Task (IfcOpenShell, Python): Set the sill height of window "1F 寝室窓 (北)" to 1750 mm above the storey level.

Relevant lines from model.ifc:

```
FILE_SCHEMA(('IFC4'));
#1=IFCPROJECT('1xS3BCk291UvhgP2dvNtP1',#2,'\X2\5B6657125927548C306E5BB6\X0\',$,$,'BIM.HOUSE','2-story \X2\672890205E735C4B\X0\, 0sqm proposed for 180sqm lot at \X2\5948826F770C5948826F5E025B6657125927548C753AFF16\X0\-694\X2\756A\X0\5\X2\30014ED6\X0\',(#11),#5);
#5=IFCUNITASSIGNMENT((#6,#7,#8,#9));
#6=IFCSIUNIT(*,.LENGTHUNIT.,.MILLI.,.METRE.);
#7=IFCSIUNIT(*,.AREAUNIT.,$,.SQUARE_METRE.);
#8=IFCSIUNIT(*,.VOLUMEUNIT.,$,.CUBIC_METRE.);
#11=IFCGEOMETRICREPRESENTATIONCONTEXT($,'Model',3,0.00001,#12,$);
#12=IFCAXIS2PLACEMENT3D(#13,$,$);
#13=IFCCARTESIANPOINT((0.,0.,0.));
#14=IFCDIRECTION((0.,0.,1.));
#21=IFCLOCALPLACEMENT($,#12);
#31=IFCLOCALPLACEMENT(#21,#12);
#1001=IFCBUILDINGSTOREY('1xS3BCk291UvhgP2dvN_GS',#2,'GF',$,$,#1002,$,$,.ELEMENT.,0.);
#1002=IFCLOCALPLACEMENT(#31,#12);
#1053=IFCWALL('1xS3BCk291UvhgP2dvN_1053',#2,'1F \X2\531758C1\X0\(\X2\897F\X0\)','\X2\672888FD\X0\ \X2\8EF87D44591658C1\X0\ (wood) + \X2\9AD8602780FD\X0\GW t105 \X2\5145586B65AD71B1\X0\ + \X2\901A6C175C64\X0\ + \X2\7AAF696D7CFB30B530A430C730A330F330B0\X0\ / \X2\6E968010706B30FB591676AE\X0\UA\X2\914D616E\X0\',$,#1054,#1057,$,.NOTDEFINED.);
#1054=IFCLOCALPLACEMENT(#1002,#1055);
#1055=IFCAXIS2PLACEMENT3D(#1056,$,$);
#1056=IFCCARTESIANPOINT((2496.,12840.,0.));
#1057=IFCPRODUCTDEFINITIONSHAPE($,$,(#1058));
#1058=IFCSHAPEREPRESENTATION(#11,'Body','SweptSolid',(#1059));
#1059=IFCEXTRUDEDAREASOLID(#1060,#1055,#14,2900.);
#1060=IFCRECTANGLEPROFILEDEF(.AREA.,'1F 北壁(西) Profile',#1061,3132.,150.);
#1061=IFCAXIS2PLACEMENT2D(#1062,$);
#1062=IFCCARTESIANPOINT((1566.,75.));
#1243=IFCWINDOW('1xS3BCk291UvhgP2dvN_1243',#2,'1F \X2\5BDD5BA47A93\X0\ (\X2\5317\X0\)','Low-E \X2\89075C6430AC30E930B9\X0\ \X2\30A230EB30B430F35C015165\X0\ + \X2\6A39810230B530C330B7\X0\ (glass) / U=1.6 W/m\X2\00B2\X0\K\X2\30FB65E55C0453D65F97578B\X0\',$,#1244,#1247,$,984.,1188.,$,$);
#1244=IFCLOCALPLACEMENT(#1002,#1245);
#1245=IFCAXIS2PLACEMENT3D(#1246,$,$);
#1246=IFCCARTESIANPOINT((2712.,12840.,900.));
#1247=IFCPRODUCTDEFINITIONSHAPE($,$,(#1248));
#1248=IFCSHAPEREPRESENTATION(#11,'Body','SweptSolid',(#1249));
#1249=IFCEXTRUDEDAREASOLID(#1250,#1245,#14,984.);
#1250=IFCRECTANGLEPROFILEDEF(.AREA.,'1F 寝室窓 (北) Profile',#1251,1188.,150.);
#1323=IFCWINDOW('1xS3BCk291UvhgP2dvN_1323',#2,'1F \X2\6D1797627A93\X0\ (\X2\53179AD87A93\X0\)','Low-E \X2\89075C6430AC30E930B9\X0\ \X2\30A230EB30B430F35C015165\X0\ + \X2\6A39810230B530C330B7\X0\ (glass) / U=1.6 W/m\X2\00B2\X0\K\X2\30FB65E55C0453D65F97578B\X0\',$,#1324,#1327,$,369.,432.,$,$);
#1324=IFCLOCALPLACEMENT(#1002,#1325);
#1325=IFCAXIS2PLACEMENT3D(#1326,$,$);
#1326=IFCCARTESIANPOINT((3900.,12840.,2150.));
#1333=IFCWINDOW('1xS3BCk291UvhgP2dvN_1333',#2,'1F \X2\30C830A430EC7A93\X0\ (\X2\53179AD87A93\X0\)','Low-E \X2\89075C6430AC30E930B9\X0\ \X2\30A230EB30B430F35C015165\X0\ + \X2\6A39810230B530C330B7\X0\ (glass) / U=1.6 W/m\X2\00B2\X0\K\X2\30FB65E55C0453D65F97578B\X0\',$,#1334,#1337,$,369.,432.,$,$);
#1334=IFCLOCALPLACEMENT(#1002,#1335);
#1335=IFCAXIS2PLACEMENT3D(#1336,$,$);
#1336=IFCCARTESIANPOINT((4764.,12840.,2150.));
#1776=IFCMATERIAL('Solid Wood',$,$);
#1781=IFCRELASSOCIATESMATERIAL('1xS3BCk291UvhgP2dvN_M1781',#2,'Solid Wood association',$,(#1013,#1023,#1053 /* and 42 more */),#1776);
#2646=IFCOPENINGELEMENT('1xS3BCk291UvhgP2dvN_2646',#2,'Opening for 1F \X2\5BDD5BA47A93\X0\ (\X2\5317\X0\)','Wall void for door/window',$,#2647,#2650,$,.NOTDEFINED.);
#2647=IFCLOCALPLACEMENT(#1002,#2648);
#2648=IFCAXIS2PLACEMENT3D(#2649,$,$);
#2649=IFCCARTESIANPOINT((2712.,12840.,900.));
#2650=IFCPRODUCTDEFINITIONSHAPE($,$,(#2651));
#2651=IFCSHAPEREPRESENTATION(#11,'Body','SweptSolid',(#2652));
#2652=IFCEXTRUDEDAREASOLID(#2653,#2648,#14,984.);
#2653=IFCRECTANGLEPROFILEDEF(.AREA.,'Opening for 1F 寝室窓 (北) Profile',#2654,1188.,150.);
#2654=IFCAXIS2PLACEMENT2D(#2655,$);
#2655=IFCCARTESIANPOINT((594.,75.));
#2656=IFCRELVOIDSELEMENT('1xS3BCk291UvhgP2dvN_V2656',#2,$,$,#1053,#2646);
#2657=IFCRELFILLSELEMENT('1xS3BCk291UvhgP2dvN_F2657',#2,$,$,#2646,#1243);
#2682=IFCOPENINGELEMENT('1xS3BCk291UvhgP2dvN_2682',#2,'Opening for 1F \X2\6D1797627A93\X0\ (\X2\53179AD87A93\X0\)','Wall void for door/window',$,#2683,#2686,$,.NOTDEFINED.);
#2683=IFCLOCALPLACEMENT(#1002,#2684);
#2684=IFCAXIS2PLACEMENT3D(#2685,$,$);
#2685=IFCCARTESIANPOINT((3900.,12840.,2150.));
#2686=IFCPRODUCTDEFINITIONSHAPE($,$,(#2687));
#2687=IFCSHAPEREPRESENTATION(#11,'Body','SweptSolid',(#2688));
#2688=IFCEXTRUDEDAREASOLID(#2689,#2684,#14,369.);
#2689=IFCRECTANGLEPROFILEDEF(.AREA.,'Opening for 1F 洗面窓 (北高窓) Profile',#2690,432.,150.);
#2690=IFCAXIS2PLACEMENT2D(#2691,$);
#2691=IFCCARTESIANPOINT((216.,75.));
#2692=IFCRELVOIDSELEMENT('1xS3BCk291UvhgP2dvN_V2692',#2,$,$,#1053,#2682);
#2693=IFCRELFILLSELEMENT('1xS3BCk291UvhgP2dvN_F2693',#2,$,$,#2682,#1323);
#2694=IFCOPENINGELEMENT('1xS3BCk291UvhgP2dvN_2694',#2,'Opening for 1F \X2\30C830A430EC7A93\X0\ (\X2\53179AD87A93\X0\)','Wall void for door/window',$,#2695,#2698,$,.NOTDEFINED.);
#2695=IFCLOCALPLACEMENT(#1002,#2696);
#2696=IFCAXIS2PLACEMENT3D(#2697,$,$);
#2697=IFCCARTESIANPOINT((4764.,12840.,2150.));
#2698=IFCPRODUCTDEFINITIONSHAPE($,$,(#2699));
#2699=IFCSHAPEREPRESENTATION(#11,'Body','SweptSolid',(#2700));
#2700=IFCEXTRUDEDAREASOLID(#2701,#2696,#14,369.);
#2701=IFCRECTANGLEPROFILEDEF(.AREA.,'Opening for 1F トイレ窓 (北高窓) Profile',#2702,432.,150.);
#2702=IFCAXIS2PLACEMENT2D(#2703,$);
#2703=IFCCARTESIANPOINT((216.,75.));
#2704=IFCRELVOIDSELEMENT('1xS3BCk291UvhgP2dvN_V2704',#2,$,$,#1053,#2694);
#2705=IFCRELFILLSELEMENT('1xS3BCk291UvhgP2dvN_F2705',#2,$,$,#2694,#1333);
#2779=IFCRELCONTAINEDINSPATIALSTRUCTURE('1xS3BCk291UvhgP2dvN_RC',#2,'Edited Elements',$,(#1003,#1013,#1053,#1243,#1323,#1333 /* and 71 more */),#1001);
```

```python
import numpy as np
import ifcopenshell
import ifcopenshell.api.geometry
import ifcopenshell.geom
import ifcopenshell.util.element
import ifcopenshell.util.placement
import ifcopenshell.util.shape
import ifcopenshell.util.unit

model = ifcopenshell.open("model.ifc")
unit_scale = ifcopenshell.util.unit.calculate_unit_scale(model)

window = model.by_guid("1xS3BCk291UvhgP2dvN_1243")
opening = window.FillsVoids[0].RelatingOpeningElement
storey = ifcopenshell.util.element.get_container(window, ifc_class="IfcBuildingStorey")
level = ifcopenshell.util.placement.get_local_placement(storey.ObjectPlacement)[2, 3]

# The opening's origin need not be at the sill, so measure its lowest point.
shape = ifcopenshell.geom.create_shape(ifcopenshell.geom.settings(), opening)
bottom = ifcopenshell.util.shape.get_shape_bottom_elevation(shape, shape.geometry) / unit_scale
dz = level + 1.75 / unit_scale - bottom

shift = np.array([0.0, 0.0, dz])
# The window is not placed relative to its opening, so move both.
for product in (opening, window):
    matrix = ifcopenshell.util.placement.get_local_placement(product.ObjectPlacement)
    matrix[:3, 3] += shift
    ifcopenshell.api.geometry.edit_object_placement(model, product=product, matrix=matrix, is_si=False)

print(f"moved by {dz * unit_scale:+.3f} m")

model.write("model_rev.ifc")
```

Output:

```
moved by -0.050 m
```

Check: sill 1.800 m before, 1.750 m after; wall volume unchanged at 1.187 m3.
